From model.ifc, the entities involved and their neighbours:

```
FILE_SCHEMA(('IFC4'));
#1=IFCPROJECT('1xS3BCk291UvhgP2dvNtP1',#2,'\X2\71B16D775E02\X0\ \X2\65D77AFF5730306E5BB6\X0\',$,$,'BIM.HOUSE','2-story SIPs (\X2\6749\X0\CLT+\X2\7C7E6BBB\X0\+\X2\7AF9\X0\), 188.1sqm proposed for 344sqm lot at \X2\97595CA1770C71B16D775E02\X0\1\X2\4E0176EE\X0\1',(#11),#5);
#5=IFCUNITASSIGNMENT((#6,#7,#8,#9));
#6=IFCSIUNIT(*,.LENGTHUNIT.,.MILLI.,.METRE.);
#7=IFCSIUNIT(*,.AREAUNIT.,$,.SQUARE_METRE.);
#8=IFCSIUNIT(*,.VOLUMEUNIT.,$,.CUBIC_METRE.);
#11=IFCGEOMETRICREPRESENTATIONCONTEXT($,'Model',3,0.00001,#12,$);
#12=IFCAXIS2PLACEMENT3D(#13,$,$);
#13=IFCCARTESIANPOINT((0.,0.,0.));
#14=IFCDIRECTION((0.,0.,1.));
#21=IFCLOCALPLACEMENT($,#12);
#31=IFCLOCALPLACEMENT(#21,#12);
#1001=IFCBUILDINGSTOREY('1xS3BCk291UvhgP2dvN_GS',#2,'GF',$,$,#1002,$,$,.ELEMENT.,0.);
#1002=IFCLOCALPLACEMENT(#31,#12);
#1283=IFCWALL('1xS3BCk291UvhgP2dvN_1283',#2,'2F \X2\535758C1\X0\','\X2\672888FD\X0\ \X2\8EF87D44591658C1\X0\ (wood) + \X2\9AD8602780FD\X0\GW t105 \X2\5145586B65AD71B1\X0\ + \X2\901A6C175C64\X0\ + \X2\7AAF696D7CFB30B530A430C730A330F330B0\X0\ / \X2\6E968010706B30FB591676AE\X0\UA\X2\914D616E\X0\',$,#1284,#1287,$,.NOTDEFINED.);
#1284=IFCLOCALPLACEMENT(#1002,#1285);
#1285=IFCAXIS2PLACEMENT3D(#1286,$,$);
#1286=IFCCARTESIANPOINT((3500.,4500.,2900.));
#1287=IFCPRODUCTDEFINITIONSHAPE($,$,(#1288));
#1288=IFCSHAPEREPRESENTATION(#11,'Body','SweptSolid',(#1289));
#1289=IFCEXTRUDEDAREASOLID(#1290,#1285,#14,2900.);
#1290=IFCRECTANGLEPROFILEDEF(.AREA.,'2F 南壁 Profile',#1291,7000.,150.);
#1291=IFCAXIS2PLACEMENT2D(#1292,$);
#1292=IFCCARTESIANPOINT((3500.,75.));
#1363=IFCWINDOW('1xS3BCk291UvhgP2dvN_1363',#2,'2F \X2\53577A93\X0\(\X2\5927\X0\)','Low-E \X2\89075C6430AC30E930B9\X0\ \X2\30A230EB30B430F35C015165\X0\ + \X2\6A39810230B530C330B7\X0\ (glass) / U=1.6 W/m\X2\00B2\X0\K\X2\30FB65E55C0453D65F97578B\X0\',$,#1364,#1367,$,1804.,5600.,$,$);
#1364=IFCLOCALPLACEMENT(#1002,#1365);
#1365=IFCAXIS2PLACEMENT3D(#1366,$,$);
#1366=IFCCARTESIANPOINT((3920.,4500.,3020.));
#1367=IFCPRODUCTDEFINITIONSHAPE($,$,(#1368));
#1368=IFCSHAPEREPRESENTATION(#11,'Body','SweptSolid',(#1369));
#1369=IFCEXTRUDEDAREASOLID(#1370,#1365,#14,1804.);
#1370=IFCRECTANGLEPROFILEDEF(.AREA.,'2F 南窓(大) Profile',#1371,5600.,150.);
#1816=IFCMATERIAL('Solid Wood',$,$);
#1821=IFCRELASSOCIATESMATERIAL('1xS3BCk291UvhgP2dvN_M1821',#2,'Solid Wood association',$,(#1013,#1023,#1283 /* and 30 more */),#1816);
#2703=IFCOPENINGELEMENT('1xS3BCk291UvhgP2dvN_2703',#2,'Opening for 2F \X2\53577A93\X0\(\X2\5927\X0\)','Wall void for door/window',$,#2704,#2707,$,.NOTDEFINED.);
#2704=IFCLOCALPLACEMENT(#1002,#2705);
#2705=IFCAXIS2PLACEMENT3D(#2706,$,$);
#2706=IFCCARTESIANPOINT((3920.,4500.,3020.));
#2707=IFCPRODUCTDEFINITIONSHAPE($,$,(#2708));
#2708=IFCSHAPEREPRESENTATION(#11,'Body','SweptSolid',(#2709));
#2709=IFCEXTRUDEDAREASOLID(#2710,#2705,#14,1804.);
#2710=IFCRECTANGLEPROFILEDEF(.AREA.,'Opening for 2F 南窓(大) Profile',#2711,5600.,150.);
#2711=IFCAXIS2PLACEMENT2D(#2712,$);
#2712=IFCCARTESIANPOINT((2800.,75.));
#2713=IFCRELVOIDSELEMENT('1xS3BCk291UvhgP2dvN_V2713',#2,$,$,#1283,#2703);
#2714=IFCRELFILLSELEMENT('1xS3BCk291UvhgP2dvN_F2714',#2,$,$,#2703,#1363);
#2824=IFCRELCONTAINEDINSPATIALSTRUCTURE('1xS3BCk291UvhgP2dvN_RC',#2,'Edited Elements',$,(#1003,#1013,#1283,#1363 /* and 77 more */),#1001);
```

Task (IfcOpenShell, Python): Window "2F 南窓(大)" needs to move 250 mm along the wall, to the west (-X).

```python
import ifcopenshell
import ifcopenshell.api.geometry
import ifcopenshell.util.placement
import ifcopenshell.util.unit

model = ifcopenshell.open("model.ifc")
unit_scale = ifcopenshell.util.unit.calculate_unit_scale(model)

window = model.by_id(1363)
opening = window.FillsVoids[0].RelatingOpeningElement
wall = opening.VoidsElements[0].RelatingBuildingElement

wall_matrix = ifcopenshell.util.placement.get_local_placement(wall.ObjectPlacement)
shift = wall_matrix[:3, 0] * -0.25 / unit_scale
before = ifcopenshell.util.placement.get_local_placement(window.ObjectPlacement)[:3, 3].copy()

# The window is not placed relative to its opening, so move both.
for product in (opening, window):
    matrix = ifcopenshell.util.placement.get_local_placement(product.ObjectPlacement)
    matrix[:3, 3] += shift
    ifcopenshell.api.geometry.edit_object_placement(model, product=product, matrix=matrix, is_si=False)

after = ifcopenshell.util.placement.get_local_placement(window.ObjectPlacement)[:3, 3]
print("window moved by", (after - before).round(3) + 0.0)

model.write("model_edited.ifc")
```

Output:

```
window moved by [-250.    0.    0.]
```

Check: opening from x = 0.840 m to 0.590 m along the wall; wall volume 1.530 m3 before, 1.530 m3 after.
